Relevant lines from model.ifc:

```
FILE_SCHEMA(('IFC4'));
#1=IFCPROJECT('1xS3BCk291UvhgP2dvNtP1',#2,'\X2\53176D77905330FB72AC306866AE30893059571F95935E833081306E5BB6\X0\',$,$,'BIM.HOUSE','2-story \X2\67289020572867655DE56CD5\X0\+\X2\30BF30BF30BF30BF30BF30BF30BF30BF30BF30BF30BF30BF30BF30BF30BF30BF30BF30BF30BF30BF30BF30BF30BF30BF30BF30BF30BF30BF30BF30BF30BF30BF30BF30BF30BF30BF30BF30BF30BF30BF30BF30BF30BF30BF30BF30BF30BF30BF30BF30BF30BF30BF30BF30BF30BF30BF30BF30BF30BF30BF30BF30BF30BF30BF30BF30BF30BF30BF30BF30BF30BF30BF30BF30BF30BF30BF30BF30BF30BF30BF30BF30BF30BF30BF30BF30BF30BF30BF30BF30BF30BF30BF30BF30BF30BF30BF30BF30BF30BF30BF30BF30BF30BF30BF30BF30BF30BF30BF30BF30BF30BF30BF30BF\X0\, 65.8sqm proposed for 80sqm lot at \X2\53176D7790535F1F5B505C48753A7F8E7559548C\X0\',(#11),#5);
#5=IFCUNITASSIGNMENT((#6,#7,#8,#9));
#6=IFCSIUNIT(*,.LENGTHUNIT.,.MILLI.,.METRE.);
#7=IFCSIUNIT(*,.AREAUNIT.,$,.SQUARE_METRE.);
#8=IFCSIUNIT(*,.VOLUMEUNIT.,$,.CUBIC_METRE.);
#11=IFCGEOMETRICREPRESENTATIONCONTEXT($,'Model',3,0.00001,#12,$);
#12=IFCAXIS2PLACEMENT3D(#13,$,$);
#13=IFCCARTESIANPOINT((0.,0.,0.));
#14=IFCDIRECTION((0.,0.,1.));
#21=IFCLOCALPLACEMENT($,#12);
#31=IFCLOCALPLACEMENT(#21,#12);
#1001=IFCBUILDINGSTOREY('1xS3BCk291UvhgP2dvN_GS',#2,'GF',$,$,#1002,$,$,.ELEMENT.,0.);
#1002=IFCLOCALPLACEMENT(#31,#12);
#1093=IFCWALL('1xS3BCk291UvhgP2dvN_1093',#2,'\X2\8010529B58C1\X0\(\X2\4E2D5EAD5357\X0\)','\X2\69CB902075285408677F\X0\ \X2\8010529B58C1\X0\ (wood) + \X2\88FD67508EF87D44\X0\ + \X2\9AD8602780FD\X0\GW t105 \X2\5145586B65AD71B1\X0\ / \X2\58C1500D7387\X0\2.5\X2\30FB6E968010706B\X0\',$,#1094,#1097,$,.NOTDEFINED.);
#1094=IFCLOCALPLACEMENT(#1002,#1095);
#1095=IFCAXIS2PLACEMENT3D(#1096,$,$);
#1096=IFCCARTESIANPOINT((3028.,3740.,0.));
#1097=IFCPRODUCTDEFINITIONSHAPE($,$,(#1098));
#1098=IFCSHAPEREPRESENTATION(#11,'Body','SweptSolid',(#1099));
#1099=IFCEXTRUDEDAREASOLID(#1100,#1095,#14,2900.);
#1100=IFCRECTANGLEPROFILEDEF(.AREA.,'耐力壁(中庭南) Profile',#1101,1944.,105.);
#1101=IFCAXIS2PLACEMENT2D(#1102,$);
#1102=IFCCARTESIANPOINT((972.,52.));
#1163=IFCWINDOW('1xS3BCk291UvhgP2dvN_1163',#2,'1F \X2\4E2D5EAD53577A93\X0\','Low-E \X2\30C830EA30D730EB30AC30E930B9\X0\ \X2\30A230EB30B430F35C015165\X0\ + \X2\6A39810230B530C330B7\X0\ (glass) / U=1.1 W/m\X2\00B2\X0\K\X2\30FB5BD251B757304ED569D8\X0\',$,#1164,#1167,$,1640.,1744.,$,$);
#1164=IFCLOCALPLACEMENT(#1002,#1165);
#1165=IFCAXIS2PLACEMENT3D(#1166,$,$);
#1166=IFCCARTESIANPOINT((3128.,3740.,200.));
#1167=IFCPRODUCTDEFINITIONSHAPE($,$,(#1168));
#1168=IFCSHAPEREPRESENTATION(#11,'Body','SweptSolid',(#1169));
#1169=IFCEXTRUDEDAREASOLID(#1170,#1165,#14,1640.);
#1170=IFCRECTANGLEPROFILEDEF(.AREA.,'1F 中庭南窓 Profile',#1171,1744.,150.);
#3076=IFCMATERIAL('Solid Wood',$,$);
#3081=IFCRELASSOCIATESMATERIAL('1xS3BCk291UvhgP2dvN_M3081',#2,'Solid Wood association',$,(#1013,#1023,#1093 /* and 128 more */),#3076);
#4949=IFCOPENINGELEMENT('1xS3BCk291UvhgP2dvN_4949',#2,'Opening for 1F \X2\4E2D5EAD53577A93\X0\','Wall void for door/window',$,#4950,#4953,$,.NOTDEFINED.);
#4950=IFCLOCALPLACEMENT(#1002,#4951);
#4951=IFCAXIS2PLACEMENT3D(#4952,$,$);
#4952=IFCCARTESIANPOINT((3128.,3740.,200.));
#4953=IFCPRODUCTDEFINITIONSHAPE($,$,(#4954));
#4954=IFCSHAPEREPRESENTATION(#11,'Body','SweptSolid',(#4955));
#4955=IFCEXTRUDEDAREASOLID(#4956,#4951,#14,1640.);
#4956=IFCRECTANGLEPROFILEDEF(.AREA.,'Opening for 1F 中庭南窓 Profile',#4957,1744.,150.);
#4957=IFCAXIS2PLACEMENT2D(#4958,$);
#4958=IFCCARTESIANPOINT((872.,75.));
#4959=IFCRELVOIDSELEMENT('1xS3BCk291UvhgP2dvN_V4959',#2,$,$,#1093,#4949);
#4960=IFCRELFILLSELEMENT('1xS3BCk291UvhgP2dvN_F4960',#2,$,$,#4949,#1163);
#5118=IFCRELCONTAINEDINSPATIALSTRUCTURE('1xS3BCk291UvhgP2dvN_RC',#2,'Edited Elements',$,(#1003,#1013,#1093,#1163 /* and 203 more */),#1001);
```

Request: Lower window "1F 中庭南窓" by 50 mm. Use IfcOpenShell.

```python
import numpy as np
import ifcopenshell
import ifcopenshell.api.geometry
import ifcopenshell.util.placement
import ifcopenshell.util.unit

model = ifcopenshell.open("model.ifc")
unit_scale = ifcopenshell.util.unit.calculate_unit_scale(model)

window = model.by_id(1163)
opening = window.FillsVoids[0].RelatingOpeningElement
dz = -0.05 / unit_scale

shift = np.array([0.0, 0.0, dz])
# The window is not placed relative to its opening, so move both.
for product in (opening, window):
    matrix = ifcopenshell.util.placement.get_local_placement(product.ObjectPlacement)
    matrix[:3, 3] += shift
    ifcopenshell.api.geometry.edit_object_placement(model, product=product, matrix=matrix, is_si=False)

print(f"moved by {dz * unit_scale:+.3f} m")

model.write("model-out.ifc")
```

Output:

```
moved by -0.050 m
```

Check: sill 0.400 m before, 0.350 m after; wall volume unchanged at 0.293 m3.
